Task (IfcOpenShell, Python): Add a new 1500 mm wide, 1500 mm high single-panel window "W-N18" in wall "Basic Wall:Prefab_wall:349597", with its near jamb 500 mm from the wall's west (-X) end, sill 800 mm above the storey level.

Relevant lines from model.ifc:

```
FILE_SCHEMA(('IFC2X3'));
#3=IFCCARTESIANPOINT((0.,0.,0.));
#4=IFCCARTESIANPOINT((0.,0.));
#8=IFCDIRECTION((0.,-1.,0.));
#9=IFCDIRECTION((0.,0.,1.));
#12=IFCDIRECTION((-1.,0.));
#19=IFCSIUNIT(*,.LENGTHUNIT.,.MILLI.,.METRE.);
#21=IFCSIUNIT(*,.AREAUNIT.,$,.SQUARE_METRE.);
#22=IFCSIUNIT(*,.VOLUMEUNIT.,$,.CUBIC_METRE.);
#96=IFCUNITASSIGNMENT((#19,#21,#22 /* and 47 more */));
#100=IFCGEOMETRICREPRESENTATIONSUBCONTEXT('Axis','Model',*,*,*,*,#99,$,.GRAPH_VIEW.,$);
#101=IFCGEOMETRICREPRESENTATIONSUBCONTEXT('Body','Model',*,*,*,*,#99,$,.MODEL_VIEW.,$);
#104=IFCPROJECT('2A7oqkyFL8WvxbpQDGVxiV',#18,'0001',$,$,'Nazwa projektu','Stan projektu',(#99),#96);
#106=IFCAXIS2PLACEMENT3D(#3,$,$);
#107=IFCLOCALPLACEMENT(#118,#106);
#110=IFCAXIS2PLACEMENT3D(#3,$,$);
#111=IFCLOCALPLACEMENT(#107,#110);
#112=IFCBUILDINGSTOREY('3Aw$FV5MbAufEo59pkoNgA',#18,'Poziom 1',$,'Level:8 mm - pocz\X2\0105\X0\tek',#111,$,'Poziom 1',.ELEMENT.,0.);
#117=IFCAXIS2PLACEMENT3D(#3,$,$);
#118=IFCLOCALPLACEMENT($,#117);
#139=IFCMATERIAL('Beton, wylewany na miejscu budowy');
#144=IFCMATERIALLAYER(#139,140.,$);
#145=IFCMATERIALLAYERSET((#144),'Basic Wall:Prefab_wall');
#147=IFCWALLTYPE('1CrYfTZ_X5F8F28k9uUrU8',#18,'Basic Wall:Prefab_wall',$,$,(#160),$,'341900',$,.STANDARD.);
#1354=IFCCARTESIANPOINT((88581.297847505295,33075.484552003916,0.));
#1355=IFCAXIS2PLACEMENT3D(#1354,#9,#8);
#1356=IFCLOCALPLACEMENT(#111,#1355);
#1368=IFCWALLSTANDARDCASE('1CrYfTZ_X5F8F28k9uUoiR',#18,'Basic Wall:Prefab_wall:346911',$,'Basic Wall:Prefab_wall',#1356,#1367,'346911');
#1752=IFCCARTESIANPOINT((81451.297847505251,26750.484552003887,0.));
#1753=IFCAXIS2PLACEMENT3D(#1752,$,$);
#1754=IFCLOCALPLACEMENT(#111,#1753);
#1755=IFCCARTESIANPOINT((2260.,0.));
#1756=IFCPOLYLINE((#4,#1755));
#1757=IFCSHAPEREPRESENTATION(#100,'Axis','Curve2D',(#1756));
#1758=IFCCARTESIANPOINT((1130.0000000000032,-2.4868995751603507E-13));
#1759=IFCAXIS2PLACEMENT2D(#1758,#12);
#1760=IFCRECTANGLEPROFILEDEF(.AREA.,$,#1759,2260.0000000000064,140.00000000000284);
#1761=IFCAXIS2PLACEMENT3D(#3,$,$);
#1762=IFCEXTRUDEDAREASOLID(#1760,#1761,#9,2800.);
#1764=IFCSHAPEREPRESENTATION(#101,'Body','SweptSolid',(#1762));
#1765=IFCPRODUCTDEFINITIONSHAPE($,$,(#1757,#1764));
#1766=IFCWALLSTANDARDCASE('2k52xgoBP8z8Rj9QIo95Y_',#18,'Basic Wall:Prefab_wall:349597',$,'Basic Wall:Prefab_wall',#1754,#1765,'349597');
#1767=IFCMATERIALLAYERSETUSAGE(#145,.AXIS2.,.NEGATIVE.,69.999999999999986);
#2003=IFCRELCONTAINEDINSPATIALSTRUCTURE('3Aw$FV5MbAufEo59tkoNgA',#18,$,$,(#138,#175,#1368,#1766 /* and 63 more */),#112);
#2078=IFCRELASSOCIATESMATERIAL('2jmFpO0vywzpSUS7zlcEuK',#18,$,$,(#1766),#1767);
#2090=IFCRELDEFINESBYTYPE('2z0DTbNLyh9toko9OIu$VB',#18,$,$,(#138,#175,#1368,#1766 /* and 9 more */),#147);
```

```python
import numpy as np
import ifcopenshell
import ifcopenshell.api.feature
import ifcopenshell.api.geometry
import ifcopenshell.api.root
import ifcopenshell.api.spatial
import ifcopenshell.api.type
import ifcopenshell.geom
import ifcopenshell.util.element
import ifcopenshell.util.placement
import ifcopenshell.util.representation
import ifcopenshell.util.shape
import ifcopenshell.util.unit

model = ifcopenshell.open("model.ifc")
unit_scale = ifcopenshell.util.unit.calculate_unit_scale(model)
settings = ifcopenshell.geom.settings()


def volume(element):
    """Net volume in cubic metres, openings subtracted."""
    shape = ifcopenshell.geom.create_shape(settings, element)
    return ifcopenshell.util.shape.get_volume(shape.geometry)


wall = model.by_guid("2k52xgoBP8z8Rj9QIo95Y_")
storey = ifcopenshell.util.element.get_container(wall, ifc_class="IfcBuildingStorey")
context = ifcopenshell.util.representation.get_context(model, "Model", "Body", "MODEL_VIEW")
before = volume(wall)

width, height, from_end, sill = 1.5, 1.5, 0.5, 0.8  # metres

# The wall runs along its own X axis, and the end named is its -X end.
wall_shape = ifcopenshell.geom.create_shape(settings, wall)
x, y, z = ifcopenshell.util.shape.get_vertices(wall_shape.geometry).T
start = x.min() + from_end
face, thickness = float(y.min()), float(y.max() - y.min())
wall_matrix = ifcopenshell.util.placement.get_local_placement(wall.ObjectPlacement)
level = ifcopenshell.util.placement.get_local_placement(storey.ObjectPlacement)[2, 3]


def in_wall(x, y):
    """Placement at x, y metres in the wall's axes, at sill height."""
    matrix = wall_matrix.copy()
    matrix[:, 3] = wall_matrix @ np.array([x / unit_scale, y / unit_scale, 0.0, 1.0])
    matrix[2, 3] = level + sill / unit_scale
    return matrix


# Opening: a box that overshoots both wall faces by 50 mm.
opening = ifcopenshell.api.root.create_entity(model, ifc_class="IfcOpeningElement")
box = ifcopenshell.api.geometry.add_wall_representation(
    model, context=context, length=width, height=height, thickness=thickness + 0.1
)
ifcopenshell.api.geometry.assign_representation(model, product=opening, representation=box)
ifcopenshell.api.geometry.edit_object_placement(model, product=opening, matrix=in_wall(start, face - 0.05), is_si=False)
ifcopenshell.api.feature.add_feature(model, feature=opening, element=wall)

window = ifcopenshell.api.root.create_entity(model, ifc_class="IfcWindow", name="W-N18")
window.OverallWidth, window.OverallHeight = width / unit_scale, height / unit_scale
body = ifcopenshell.api.geometry.add_window_representation(
    model,
    context=context,
    overall_width=window.OverallWidth,
    overall_height=window.OverallHeight,
    partition_type="SINGLE_PANEL",
)
ifcopenshell.api.geometry.assign_representation(model, product=window, representation=body)
ifcopenshell.api.spatial.assign_container(model, products=[window], relating_structure=storey)
fills = ifcopenshell.api.feature.add_filling(model, opening=opening, element=window)
fills.OwnerHistory = window.OwnerHistory  # required in IFC2X3

# IFC2X3 keeps the operation on the window style.
style = ifcopenshell.api.root.create_entity(model, ifc_class="IfcWindowStyle", name="W-N18")
style.OperationType, style.ConstructionType = "SINGLE_PANEL", "NOTDEFINED"
style.ParameterTakesPrecedence = style.Sizeable = False
ifcopenshell.api.type.assign_type(model, related_objects=[window], relating_type=style)

# Centre the window in the wall's thickness.
ifcopenshell.api.geometry.edit_object_placement(model, product=window, matrix=in_wall(start, face), is_si=False)
window_shape = ifcopenshell.geom.create_shape(settings, window)
depth = ifcopenshell.util.shape.get_vertices(window_shape.geometry)[:, 1]
offset = face + thickness / 2 - (depth.min() + depth.max()) / 2
ifcopenshell.api.geometry.edit_object_placement(model, product=window, matrix=in_wall(start, offset), is_si=False)

after = volume(wall)

print(f"wall volume {before:.3f} -> {after:.3f} m3")

model.write("model_rev.ifc")
```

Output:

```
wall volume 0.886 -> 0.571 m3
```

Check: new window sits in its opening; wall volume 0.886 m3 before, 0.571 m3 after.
